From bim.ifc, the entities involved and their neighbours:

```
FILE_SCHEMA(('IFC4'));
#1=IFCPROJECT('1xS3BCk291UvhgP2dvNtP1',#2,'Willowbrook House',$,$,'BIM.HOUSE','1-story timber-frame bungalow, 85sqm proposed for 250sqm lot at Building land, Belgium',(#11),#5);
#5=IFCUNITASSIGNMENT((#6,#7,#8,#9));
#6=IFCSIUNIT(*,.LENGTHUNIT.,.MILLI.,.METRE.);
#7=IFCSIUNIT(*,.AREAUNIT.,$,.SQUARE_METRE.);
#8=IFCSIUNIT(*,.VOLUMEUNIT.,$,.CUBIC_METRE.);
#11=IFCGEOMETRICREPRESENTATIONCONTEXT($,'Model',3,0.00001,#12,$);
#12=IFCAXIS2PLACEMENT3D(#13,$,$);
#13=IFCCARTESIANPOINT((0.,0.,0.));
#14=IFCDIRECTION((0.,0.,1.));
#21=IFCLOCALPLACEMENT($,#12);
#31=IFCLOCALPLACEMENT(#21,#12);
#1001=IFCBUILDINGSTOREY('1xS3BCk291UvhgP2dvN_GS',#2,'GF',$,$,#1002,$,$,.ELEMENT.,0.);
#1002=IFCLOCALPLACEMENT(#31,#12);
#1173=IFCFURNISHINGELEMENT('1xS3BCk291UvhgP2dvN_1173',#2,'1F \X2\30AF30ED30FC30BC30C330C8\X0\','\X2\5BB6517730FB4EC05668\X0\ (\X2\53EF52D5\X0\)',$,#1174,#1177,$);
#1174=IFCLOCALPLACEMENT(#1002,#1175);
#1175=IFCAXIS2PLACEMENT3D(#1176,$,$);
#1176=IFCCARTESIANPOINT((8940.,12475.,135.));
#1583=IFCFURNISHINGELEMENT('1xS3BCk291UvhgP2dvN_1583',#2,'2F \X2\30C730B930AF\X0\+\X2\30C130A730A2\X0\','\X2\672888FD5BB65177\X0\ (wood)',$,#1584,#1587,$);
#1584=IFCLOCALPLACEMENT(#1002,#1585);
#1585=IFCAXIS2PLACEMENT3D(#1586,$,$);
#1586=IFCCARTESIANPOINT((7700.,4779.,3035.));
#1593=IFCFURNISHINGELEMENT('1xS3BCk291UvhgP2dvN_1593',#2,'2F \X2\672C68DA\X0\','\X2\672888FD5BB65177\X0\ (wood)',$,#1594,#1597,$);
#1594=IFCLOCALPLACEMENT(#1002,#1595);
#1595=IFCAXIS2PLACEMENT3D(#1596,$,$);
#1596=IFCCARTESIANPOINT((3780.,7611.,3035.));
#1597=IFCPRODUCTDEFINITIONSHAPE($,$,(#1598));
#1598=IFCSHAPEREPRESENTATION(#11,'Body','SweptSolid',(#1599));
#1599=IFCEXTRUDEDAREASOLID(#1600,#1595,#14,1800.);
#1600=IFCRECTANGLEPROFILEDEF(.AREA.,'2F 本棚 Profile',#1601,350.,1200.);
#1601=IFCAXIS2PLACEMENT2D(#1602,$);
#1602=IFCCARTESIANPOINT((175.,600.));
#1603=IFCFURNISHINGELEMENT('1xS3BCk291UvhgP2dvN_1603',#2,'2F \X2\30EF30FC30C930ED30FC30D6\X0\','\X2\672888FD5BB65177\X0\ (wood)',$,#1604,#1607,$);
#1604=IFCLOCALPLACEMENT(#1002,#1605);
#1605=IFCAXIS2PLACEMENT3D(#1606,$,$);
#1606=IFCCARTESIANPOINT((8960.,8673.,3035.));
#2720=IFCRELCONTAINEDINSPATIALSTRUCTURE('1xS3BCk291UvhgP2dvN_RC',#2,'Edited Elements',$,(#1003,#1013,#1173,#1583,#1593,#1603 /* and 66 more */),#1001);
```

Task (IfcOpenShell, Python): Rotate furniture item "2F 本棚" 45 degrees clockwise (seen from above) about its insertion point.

```python
import ifcopenshell
import ifcopenshell.api.geometry
import ifcopenshell.util.placement

model = ifcopenshell.open("bim.ifc")

item = model.by_guid("1xS3BCk291UvhgP2dvN_1593")
matrix = ifcopenshell.util.placement.get_local_placement(item.ObjectPlacement)
matrix = matrix @ ifcopenshell.util.placement.rotation(-45, "Z")
ifcopenshell.api.geometry.edit_object_placement(model, product=item, matrix=matrix, is_si=False)

print(ifcopenshell.util.placement.get_local_placement(item.ObjectPlacement).round(3) + 0.0)

model.write("bim_edited.ifc")
```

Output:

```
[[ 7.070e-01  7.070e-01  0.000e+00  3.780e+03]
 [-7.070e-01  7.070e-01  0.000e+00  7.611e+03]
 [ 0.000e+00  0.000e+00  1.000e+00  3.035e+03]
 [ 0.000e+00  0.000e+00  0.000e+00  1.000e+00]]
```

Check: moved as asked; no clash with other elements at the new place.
